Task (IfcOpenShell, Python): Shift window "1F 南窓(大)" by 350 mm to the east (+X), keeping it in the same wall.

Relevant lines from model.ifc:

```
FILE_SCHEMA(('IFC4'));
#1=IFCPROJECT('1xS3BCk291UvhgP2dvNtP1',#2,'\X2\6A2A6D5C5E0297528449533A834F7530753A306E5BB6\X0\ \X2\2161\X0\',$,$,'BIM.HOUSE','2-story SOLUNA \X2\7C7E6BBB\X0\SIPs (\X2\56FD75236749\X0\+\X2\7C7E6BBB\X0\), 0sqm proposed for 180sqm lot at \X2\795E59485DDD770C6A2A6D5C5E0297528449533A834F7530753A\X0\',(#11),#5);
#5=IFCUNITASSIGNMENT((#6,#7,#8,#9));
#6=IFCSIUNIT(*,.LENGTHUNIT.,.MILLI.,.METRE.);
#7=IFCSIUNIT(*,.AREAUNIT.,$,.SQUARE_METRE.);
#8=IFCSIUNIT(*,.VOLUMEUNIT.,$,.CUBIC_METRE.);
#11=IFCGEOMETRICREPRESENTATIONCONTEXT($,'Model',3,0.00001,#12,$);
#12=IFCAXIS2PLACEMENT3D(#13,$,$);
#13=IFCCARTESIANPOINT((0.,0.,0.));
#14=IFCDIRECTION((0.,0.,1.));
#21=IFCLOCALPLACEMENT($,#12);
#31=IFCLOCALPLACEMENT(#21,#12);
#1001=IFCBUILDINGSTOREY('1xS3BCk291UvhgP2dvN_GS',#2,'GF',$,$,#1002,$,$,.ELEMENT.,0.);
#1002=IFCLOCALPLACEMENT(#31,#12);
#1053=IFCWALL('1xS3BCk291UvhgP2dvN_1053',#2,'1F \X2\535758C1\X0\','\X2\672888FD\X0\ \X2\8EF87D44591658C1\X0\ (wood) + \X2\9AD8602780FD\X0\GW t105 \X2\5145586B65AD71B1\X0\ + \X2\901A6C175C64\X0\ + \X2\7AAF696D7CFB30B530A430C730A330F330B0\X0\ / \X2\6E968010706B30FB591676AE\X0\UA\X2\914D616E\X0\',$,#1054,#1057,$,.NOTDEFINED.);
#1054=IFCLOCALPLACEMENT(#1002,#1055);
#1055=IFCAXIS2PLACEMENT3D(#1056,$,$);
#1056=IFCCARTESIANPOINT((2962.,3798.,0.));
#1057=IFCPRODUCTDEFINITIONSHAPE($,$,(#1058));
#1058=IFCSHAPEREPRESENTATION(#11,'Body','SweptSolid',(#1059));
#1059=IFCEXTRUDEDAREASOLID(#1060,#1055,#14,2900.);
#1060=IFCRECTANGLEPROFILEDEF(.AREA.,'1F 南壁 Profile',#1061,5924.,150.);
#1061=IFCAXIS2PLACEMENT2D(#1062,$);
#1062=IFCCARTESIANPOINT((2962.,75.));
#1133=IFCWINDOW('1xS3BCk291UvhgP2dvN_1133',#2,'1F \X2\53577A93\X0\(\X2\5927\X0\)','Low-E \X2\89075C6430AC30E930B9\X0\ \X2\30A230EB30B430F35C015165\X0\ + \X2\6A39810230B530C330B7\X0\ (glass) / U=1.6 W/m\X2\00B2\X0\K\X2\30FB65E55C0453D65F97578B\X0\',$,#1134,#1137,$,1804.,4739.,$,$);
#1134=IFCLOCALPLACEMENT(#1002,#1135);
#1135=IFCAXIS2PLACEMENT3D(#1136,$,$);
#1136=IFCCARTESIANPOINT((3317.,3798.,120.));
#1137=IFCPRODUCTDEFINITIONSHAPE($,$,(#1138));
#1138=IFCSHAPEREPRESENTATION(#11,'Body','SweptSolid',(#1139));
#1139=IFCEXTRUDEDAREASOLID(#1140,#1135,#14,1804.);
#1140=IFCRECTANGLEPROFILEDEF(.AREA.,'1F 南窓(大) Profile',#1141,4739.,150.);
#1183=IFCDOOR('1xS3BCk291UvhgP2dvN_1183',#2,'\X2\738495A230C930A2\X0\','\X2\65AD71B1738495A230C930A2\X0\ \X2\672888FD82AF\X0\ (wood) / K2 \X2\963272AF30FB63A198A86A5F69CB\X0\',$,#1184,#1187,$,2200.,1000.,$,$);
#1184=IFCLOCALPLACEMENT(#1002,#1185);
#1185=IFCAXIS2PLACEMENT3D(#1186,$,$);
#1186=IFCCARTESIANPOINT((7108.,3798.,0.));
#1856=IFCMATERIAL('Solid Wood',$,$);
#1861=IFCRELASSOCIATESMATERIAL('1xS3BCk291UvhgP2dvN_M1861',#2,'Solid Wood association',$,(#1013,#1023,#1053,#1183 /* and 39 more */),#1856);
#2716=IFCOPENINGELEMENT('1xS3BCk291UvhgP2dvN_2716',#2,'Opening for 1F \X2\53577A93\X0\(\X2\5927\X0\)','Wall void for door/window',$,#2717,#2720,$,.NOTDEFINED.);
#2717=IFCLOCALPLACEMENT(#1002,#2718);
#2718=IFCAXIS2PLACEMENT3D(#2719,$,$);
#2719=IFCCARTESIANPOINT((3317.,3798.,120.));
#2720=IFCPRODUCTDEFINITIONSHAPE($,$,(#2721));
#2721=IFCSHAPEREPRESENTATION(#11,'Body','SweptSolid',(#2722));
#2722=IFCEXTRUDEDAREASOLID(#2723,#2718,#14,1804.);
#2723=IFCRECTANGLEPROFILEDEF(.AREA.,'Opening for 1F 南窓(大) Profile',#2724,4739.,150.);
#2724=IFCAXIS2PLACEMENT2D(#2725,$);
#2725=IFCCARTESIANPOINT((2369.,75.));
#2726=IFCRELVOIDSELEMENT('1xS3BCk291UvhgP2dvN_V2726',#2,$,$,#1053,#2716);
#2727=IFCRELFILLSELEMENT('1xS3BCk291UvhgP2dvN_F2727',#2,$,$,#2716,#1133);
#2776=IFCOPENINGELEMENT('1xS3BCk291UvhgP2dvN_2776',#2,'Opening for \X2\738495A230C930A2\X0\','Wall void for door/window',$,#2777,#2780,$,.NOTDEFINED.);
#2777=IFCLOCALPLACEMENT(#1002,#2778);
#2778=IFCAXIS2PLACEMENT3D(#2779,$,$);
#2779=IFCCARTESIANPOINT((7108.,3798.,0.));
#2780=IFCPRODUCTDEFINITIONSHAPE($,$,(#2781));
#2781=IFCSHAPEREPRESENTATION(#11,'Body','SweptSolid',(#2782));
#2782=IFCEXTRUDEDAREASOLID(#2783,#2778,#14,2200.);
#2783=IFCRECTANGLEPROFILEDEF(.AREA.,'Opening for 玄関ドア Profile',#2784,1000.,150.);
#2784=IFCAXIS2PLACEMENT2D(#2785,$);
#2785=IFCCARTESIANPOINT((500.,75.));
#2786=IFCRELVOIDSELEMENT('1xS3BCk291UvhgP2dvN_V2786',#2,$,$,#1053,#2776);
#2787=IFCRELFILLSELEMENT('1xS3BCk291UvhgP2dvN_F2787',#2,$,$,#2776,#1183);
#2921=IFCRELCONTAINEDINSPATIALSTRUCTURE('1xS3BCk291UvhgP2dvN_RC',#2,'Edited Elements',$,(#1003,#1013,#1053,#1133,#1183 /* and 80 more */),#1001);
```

```python
import ifcopenshell
import ifcopenshell.api.geometry
import ifcopenshell.util.placement

model = ifcopenshell.open("model.ifc")

window = model.by_id(1133)
opening = window.FillsVoids[0].RelatingOpeningElement
wall = opening.VoidsElements[0].RelatingBuildingElement

wall_matrix = ifcopenshell.util.placement.get_local_placement(wall.ObjectPlacement)
shift = wall_matrix[:3, 0] * 350.0
before = ifcopenshell.util.placement.get_local_placement(window.ObjectPlacement)[:3, 3].copy()

# The window is not placed relative to its opening, so move both.
for product in (opening, window):
    matrix = ifcopenshell.util.placement.get_local_placement(product.ObjectPlacement)
    matrix[:3, 3] += shift
    ifcopenshell.api.geometry.edit_object_placement(model, product=product, matrix=matrix, is_si=False)

after = ifcopenshell.util.placement.get_local_placement(window.ObjectPlacement)[:3, 3]
print("window moved by", (after - before).round(3) + 0.0)

model.write("model_edited.ifc")
```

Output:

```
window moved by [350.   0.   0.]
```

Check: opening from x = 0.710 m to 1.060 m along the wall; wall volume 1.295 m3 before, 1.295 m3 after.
